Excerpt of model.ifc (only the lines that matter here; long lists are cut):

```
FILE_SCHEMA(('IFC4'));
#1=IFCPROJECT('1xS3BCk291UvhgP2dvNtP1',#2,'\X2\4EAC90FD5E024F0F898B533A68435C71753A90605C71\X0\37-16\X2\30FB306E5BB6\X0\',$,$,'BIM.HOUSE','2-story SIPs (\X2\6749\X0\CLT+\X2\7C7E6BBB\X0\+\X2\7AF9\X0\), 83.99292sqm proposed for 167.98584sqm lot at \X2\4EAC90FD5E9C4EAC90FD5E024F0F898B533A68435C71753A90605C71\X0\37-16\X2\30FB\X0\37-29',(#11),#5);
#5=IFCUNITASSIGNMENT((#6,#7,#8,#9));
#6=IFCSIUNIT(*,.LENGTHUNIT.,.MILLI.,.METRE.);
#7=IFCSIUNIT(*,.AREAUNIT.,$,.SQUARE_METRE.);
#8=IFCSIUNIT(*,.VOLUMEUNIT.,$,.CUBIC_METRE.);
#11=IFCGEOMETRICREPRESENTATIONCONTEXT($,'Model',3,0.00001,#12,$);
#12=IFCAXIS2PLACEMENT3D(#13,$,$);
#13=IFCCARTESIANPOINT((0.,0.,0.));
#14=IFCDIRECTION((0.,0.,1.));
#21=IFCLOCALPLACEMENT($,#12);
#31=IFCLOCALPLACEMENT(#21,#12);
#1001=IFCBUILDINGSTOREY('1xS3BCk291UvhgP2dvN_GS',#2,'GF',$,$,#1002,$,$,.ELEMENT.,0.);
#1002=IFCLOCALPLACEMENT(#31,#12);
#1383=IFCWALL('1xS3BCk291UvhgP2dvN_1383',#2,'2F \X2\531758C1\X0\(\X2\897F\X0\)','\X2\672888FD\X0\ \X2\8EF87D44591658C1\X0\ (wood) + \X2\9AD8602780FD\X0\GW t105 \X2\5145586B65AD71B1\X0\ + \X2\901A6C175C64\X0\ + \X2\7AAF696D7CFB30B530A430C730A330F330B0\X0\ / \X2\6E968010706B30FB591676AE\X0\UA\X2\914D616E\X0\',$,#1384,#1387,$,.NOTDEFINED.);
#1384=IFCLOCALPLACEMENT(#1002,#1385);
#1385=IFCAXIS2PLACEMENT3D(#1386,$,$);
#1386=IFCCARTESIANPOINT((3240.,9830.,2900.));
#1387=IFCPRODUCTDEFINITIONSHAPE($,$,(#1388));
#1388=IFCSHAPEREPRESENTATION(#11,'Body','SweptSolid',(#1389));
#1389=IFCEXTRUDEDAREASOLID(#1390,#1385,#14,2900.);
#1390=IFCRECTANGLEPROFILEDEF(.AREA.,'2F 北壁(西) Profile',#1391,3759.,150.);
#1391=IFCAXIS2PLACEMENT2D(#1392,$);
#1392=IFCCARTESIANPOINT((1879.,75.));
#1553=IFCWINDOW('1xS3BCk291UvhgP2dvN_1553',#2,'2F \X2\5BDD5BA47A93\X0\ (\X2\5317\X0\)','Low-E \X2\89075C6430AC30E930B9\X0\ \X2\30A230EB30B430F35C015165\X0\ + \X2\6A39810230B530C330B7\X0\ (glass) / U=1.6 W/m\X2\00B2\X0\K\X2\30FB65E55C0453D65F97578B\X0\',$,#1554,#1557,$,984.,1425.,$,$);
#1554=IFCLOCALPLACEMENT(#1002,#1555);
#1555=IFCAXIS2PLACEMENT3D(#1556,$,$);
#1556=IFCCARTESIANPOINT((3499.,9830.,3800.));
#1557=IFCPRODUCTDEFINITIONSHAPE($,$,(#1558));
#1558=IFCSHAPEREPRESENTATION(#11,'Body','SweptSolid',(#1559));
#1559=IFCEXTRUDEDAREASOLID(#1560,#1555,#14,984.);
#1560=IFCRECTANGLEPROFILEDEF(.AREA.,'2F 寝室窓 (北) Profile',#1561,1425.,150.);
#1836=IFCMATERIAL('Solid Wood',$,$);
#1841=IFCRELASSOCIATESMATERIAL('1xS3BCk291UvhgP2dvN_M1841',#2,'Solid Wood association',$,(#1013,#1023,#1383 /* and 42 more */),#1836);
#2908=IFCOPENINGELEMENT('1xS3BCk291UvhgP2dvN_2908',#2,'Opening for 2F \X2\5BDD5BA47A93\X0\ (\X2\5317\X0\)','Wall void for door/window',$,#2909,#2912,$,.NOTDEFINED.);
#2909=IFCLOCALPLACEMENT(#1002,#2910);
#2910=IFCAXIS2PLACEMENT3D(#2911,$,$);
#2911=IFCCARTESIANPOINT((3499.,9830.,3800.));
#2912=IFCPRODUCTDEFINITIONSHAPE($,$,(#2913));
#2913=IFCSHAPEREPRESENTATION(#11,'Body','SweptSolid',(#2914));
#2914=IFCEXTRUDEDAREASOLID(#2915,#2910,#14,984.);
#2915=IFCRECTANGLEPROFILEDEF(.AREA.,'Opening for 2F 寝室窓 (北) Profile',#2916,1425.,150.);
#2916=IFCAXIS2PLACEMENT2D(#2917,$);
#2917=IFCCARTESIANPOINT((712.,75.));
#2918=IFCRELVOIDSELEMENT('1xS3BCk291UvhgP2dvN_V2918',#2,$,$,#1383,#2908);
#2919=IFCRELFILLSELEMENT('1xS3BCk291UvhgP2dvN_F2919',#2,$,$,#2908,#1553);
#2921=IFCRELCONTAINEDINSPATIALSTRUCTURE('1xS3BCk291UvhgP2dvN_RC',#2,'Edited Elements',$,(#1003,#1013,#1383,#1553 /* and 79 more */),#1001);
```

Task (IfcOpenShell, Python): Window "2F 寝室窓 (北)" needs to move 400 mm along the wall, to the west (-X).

```python
import ifcopenshell
import ifcopenshell.api.geometry
import ifcopenshell.util.placement
import ifcopenshell.util.unit

model = ifcopenshell.open("model.ifc")
unit_scale = ifcopenshell.util.unit.calculate_unit_scale(model)

window = model.by_guid("1xS3BCk291UvhgP2dvN_1553")
opening = window.FillsVoids[0].RelatingOpeningElement
wall = opening.VoidsElements[0].RelatingBuildingElement

wall_matrix = ifcopenshell.util.placement.get_local_placement(wall.ObjectPlacement)
shift = wall_matrix[:3, 0] * -0.4 / unit_scale
before = ifcopenshell.util.placement.get_local_placement(window.ObjectPlacement)[:3, 3].copy()

# The window is not placed relative to its opening, so move both.
for product in (opening, window):
    matrix = ifcopenshell.util.placement.get_local_placement(product.ObjectPlacement)
    matrix[:3, 3] += shift
    ifcopenshell.api.geometry.edit_object_placement(model, product=product, matrix=matrix, is_si=False)

after = ifcopenshell.util.placement.get_local_placement(window.ObjectPlacement)[:3, 3]
print("window moved by", (after - before).round(3) + 0.0)

model.write("model-out.ifc")
```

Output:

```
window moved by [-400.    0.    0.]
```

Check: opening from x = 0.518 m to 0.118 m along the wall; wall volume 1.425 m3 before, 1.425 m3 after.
